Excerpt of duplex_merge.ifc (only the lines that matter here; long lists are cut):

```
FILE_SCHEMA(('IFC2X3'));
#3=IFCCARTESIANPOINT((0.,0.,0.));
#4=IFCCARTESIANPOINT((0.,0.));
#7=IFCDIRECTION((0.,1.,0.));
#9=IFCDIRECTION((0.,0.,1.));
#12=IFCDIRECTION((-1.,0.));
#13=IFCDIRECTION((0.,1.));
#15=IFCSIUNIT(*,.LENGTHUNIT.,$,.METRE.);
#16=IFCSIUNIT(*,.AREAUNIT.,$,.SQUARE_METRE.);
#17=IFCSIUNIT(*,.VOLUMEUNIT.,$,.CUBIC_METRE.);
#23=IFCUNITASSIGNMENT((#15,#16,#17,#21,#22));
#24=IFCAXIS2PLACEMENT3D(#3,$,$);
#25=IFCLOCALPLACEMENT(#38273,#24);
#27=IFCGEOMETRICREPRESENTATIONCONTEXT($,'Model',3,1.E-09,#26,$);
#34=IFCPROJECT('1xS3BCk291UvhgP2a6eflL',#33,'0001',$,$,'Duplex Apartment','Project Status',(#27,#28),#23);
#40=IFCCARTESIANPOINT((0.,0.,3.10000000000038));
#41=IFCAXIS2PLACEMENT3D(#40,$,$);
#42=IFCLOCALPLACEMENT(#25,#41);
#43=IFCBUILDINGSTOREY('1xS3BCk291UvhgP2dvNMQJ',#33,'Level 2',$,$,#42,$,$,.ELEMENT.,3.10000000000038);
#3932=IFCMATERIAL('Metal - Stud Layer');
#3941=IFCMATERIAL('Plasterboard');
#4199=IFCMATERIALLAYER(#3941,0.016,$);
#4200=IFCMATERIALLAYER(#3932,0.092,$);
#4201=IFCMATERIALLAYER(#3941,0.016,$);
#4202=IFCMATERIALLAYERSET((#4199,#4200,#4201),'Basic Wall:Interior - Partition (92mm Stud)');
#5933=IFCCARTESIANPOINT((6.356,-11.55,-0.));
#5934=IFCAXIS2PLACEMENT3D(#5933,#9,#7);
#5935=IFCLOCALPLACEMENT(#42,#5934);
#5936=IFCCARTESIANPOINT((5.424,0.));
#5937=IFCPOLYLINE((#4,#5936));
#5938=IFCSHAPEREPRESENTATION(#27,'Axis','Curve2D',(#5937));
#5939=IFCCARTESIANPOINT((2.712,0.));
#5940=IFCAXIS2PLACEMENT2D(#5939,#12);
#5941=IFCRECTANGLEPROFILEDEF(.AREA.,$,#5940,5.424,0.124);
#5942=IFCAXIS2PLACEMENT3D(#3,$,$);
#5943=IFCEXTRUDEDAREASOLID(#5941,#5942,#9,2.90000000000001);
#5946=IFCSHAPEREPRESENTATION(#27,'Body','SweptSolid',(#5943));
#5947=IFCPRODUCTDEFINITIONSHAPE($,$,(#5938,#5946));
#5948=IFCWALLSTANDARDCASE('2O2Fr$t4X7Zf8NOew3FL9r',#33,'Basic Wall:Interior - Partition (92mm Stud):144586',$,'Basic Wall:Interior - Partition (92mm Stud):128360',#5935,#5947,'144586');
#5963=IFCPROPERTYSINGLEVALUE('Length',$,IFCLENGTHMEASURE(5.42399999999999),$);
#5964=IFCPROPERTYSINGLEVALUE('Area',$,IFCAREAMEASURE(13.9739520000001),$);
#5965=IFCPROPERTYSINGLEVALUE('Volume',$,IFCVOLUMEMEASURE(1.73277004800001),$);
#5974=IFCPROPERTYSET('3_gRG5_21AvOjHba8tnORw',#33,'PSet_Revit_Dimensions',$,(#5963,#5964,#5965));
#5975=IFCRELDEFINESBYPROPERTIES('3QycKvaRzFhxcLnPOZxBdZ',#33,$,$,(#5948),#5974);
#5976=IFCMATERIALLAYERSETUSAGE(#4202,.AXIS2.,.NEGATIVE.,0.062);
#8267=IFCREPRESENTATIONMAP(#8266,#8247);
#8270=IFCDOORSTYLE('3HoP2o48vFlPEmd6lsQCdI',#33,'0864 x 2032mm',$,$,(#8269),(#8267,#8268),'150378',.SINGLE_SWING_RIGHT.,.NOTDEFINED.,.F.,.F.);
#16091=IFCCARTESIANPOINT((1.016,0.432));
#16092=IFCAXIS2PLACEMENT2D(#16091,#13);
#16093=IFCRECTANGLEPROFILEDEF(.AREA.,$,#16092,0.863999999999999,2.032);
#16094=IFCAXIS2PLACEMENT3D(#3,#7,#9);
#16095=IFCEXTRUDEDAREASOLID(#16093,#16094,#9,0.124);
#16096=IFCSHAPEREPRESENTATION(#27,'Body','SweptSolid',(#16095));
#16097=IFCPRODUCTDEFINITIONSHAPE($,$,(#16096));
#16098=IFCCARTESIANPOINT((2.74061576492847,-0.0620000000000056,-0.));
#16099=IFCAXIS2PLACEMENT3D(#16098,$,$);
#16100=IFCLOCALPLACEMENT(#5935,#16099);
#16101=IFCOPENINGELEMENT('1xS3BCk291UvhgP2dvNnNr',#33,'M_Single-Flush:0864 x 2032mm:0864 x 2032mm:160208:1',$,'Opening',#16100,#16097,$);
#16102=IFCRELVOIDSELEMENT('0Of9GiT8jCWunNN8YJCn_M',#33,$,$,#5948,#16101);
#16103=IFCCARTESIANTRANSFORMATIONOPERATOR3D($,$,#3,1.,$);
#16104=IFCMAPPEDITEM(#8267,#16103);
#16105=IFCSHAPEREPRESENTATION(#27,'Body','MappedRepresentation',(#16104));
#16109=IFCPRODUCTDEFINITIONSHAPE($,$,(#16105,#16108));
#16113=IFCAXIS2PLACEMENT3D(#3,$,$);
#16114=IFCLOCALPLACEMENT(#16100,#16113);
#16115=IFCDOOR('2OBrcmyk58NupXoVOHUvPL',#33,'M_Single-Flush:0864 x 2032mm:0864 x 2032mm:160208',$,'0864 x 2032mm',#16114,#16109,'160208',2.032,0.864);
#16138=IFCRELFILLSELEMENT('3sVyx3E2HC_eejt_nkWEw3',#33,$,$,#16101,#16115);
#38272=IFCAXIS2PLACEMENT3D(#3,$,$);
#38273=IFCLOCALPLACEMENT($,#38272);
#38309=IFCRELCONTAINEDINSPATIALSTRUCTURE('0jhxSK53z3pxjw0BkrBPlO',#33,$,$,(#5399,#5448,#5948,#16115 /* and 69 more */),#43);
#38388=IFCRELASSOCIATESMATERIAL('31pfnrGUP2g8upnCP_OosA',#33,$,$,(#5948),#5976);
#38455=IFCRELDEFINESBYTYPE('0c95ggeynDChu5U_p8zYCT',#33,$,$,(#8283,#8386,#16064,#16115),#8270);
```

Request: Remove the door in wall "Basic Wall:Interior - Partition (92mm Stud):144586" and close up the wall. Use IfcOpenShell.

```python
import ifcopenshell
import ifcopenshell.api.feature
import ifcopenshell.api.pset
import ifcopenshell.api.root
import ifcopenshell.geom
import ifcopenshell.util.element
import ifcopenshell.util.shape
import ifcopenshell.util.unit

model = ifcopenshell.open("duplex_merge.ifc")
area_scale = ifcopenshell.util.unit.calculate_unit_scale(model, "AREAUNIT")
volume_scale = ifcopenshell.util.unit.calculate_unit_scale(model, "VOLUMEUNIT")
settings = ifcopenshell.geom.settings()


def volume(element):
    """Net volume in cubic metres, openings subtracted."""
    shape = ifcopenshell.geom.create_shape(settings, element)
    return ifcopenshell.util.shape.get_volume(shape.geometry)


door = model.by_id(16115)
opening = door.FillsVoids[0].RelatingOpeningElement
wall = opening.VoidsElements[0].RelatingBuildingElement
before = volume(wall)

ifcopenshell.api.root.remove_product(model, product=door)
ifcopenshell.api.feature.remove_feature(model, feature=opening)

after = volume(wall)
thickness = 0.124  # wall thickness in metres

# Update the wall's stored quantities.
pset = model.by_id(ifcopenshell.util.element.get_pset(wall, "PSet_Revit_Dimensions", should_inherit=False)["id"])
ifcopenshell.api.pset.edit_pset(model, pset=pset, properties={
    "Area": model.create_entity("IfcAreaMeasure", after / thickness / area_scale),
    "Volume": model.create_entity("IfcVolumeMeasure", after / volume_scale),
})

print(f"wall volume {before:.3f} -> {after:.3f} m3")

model.write("duplex_merge-out.ifc")
```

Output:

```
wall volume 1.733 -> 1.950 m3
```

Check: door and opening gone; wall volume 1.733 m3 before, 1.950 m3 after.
